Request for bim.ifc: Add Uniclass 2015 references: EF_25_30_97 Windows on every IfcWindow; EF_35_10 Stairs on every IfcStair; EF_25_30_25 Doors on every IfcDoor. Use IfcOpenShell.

First a look at what the model holds.

```python
import ifcopenshell

model = ifcopenshell.open("bim.ifc")
print(model.schema)
print("classifications:", [c.Name for c in model.by_type("IfcClassification")])
for ifc_class in ("IfcDoor", "IfcRoof", "IfcStair", "IfcWall", "IfcWindow"):
    print(ifc_class, len(model.by_type(ifc_class)))
```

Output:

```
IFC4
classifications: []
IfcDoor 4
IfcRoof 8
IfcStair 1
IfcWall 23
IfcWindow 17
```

```python
import ifcopenshell
import ifcopenshell.api.classification

model = ifcopenshell.open("bim.ifc")

system = ifcopenshell.api.classification.add_classification(model, classification="Uniclass 2015")

codes = {
    "IfcWindow": ("EF_25_30_97", "Windows"),
    "IfcStair": ("EF_35_10", "Stairs"),
    "IfcDoor": ("EF_25_30_25", "Doors"),
}
for ifc_class, (code, name) in codes.items():
    products = model.by_type(ifc_class)
    ifcopenshell.api.classification.add_reference(
        model, products=products, classification=system, identification=code, name=name
    )
    print(code, len(products))

model.write("bim_rev.ifc")
```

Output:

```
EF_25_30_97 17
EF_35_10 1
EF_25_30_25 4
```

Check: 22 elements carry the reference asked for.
